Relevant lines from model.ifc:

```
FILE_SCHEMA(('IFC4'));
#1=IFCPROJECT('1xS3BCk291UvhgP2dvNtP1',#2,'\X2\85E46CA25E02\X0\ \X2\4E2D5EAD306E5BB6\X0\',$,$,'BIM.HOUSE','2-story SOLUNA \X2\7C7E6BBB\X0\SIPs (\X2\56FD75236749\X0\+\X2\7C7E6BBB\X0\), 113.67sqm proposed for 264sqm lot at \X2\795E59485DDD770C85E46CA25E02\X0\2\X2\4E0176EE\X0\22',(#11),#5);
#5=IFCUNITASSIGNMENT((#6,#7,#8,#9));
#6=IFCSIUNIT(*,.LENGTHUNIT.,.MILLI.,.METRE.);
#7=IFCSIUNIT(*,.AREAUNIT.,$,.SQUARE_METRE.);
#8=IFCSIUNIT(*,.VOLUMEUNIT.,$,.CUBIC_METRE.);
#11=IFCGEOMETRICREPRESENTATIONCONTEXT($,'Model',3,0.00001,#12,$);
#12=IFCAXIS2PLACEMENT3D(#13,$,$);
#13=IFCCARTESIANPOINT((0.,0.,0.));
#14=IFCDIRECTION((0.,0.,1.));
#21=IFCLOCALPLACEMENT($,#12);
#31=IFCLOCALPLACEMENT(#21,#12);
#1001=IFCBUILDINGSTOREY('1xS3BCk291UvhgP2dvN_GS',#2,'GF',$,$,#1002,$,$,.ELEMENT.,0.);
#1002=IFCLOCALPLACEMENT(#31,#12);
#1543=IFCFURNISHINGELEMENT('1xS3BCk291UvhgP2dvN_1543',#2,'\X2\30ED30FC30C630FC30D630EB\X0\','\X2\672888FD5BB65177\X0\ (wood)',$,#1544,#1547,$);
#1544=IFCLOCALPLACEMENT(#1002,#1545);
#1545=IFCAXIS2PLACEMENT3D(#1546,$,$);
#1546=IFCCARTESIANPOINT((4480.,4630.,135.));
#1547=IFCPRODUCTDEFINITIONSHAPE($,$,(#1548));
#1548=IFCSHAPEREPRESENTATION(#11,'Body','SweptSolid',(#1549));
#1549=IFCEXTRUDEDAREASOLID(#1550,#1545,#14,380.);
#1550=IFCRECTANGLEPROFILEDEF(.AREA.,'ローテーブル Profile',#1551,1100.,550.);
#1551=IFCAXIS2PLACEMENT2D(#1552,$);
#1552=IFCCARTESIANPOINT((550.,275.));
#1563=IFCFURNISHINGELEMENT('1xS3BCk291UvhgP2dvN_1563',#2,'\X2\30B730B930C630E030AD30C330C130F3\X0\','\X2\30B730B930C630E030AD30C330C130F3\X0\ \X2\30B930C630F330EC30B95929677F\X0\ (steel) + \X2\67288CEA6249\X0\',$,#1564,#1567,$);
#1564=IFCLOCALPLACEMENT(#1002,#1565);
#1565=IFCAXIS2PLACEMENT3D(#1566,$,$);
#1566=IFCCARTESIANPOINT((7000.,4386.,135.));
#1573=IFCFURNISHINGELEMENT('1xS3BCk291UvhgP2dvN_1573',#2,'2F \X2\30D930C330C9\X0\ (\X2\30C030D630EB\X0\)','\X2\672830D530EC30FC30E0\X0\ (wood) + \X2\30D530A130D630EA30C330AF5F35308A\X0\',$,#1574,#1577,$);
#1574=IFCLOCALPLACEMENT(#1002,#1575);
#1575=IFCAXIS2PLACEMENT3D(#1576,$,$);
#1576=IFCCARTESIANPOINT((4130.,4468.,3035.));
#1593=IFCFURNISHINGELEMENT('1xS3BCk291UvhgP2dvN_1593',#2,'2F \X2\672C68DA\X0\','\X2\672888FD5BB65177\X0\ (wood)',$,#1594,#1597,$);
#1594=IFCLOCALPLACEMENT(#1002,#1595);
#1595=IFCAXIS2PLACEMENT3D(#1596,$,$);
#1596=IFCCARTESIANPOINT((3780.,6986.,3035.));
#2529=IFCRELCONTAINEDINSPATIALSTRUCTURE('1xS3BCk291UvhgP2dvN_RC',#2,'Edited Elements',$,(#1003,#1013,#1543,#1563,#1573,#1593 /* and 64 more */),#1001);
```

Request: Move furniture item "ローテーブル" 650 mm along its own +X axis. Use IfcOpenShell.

```python
import ifcopenshell
import ifcopenshell.api.geometry
import ifcopenshell.util.placement

model = ifcopenshell.open("model.ifc")

item = model.by_guid("1xS3BCk291UvhgP2dvN_1543")
matrix = ifcopenshell.util.placement.get_local_placement(item.ObjectPlacement)
matrix[:3, 3] += matrix[:3, 0] * 650.0
ifcopenshell.api.geometry.edit_object_placement(model, product=item, matrix=matrix, is_si=False)

print(ifcopenshell.util.placement.get_local_placement(item.ObjectPlacement).round(3) + 0.0)

model.write("model_edited.ifc")
```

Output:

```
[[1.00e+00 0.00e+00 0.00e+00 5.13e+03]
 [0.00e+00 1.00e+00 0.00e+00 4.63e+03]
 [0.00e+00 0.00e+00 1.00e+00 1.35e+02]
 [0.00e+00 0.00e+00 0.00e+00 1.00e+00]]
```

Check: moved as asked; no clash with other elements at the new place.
